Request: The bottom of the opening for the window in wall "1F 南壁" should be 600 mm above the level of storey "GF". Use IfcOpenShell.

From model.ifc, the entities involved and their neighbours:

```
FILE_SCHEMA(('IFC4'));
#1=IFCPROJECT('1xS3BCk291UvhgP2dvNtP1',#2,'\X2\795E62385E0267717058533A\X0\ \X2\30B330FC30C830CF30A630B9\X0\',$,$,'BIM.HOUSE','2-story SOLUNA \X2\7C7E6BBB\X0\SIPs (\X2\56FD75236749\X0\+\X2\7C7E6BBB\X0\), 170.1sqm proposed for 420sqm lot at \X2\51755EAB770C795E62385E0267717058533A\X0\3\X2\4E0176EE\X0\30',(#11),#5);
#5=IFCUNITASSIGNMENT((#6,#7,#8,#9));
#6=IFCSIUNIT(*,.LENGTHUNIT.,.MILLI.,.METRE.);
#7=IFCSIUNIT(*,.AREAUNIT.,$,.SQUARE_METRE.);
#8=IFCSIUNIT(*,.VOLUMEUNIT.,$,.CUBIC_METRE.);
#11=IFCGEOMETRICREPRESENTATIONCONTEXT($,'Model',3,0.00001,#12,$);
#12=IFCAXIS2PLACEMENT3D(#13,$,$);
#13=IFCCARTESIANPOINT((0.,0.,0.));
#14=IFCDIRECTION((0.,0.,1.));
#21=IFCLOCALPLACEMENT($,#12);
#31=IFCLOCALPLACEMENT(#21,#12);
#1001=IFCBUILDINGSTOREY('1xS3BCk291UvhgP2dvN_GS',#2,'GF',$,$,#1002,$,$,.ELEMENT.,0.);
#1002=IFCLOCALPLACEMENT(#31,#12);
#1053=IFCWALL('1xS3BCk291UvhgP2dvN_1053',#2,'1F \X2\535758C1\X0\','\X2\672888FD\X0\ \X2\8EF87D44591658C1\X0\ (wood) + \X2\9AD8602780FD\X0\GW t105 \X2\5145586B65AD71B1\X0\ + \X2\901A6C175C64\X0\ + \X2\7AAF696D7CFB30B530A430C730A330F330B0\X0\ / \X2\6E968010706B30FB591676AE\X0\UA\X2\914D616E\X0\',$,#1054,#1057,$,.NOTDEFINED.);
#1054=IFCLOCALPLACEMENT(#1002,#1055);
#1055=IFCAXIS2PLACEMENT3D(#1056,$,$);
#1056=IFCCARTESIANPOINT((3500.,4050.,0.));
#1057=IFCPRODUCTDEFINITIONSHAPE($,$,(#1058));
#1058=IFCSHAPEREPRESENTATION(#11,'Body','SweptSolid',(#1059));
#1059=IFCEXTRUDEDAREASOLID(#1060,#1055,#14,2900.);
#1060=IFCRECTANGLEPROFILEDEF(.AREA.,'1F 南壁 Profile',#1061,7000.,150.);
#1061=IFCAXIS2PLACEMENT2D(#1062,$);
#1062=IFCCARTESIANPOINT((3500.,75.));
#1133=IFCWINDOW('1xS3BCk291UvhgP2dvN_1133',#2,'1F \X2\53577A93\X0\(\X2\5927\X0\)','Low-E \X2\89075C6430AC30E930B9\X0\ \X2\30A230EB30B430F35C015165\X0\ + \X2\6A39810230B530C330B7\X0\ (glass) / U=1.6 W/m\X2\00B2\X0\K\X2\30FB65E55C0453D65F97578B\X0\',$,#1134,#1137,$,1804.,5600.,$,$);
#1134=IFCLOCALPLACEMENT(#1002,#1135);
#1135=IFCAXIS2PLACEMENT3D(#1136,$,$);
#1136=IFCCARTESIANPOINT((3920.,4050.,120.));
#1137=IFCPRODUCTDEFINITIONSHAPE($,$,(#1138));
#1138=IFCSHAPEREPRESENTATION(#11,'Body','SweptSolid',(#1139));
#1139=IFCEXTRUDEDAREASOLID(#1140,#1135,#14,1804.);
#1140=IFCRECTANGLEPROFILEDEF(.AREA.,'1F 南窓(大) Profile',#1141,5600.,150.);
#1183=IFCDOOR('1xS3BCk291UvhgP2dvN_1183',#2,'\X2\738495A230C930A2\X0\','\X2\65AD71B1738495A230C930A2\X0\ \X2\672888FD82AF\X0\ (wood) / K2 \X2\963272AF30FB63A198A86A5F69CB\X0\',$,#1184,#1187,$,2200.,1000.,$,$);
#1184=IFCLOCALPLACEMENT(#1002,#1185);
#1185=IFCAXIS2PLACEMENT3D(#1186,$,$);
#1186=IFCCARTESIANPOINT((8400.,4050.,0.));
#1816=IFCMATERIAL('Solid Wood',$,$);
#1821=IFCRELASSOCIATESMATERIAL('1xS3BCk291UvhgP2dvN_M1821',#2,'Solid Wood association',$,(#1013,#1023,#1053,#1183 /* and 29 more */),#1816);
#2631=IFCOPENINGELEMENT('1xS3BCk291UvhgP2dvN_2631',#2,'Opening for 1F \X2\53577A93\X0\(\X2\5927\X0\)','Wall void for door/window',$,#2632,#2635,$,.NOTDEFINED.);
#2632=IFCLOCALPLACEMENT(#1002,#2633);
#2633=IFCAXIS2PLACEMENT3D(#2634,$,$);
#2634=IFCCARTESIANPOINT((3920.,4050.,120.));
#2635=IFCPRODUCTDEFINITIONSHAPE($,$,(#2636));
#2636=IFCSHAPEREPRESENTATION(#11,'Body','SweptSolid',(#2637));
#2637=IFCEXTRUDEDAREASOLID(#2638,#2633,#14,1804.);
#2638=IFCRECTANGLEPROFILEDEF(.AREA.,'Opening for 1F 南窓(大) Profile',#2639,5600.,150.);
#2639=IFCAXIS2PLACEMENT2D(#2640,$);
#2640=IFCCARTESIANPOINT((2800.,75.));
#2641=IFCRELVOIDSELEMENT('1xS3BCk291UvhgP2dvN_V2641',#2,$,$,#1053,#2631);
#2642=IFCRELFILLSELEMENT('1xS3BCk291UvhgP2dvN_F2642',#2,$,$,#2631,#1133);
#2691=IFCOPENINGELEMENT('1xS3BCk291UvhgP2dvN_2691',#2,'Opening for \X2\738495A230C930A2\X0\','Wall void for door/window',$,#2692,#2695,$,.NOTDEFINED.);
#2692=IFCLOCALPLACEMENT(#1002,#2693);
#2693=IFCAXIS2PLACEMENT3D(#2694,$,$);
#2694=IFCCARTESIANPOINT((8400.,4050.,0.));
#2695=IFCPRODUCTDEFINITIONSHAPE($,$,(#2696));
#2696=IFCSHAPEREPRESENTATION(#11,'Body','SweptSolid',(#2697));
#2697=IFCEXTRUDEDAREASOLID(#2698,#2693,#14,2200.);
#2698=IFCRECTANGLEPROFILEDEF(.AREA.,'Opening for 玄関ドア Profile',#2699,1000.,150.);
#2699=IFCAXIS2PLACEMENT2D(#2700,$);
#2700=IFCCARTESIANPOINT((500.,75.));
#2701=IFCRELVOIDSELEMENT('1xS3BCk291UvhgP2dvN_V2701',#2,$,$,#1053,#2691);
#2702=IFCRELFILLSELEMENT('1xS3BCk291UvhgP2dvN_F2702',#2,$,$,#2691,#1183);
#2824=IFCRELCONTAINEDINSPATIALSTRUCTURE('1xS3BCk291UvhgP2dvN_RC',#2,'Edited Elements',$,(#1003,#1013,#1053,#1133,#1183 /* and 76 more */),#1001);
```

```python
import numpy as np
import ifcopenshell
import ifcopenshell.api.geometry
import ifcopenshell.geom
import ifcopenshell.util.element
import ifcopenshell.util.placement
import ifcopenshell.util.shape
import ifcopenshell.util.unit

model = ifcopenshell.open("model.ifc")
unit_scale = ifcopenshell.util.unit.calculate_unit_scale(model)

window = model.by_guid("1xS3BCk291UvhgP2dvN_1133")
opening = window.FillsVoids[0].RelatingOpeningElement
storey = ifcopenshell.util.element.get_container(window, ifc_class="IfcBuildingStorey")
level = ifcopenshell.util.placement.get_local_placement(storey.ObjectPlacement)[2, 3]

# The opening's origin need not be at the sill, so measure its lowest point.
shape = ifcopenshell.geom.create_shape(ifcopenshell.geom.settings(), opening)
bottom = ifcopenshell.util.shape.get_shape_bottom_elevation(shape, shape.geometry) / unit_scale
dz = level + 0.6 / unit_scale - bottom

shift = np.array([0.0, 0.0, dz])
# The window is not placed relative to its opening, so move both.
for product in (opening, window):
    matrix = ifcopenshell.util.placement.get_local_placement(product.ObjectPlacement)
    matrix[:3, 3] += shift
    ifcopenshell.api.geometry.edit_object_placement(model, product=product, matrix=matrix, is_si=False)

print(f"moved by {dz * unit_scale:+.3f} m")

model.write("model_v2.ifc")
```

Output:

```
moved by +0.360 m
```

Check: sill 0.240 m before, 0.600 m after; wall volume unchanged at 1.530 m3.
